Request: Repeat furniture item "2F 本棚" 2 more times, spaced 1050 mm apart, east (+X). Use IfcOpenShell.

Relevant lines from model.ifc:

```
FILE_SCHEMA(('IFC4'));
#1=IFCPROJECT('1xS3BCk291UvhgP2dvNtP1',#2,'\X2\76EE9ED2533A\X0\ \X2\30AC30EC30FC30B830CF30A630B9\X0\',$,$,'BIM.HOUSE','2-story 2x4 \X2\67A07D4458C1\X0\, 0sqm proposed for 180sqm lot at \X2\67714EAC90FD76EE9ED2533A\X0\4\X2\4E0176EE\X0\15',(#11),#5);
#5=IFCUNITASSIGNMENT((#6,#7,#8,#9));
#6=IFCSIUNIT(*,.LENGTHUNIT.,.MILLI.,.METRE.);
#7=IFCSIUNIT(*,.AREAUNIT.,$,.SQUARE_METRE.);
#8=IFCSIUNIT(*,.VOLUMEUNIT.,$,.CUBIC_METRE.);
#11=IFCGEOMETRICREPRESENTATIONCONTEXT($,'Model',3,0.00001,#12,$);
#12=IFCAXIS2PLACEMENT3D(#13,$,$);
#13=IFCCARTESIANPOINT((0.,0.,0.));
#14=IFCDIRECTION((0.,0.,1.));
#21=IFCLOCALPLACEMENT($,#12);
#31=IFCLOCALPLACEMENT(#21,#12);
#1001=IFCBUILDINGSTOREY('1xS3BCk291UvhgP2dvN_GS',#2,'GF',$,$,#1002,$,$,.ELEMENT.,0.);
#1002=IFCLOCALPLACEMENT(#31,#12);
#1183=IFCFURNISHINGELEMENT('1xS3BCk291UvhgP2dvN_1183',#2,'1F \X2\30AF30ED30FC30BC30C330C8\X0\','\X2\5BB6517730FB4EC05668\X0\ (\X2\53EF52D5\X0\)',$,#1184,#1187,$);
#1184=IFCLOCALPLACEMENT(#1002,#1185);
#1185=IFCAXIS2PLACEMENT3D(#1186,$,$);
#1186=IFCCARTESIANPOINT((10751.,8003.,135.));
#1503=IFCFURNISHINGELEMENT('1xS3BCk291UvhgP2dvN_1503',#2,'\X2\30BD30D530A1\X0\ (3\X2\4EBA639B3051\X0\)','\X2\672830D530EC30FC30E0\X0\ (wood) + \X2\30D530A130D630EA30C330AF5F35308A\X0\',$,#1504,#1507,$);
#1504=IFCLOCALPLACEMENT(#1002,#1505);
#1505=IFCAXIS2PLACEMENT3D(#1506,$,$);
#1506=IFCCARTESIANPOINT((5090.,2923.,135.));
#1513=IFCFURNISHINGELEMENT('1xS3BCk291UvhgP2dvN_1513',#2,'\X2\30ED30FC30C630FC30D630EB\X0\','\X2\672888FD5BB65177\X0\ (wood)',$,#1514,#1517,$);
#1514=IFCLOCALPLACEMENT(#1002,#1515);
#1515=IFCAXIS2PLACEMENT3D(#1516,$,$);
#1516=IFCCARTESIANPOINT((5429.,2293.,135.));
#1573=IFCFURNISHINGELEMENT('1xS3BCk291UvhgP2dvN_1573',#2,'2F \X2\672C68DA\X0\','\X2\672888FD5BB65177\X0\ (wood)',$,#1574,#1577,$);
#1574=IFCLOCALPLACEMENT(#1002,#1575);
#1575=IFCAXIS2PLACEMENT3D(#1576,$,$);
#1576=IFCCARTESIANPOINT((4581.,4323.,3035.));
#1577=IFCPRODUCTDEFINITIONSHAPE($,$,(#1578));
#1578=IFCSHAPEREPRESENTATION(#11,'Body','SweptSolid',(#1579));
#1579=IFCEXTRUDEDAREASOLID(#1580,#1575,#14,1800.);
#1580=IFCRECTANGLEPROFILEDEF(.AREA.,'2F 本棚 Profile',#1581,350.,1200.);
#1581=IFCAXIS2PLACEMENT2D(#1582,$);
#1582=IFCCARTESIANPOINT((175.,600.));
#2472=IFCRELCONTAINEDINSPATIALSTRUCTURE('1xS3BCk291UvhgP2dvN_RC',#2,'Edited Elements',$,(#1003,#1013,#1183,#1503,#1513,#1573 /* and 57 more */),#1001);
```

```python
import numpy as np
import ifcopenshell
import ifcopenshell.api.geometry
import ifcopenshell.api.root
import ifcopenshell.util.element
import ifcopenshell.util.placement

model = ifcopenshell.open("model.ifc")


def reuse_history(source, copy):
    """copy_class also copies each property set's owner history, people and application; keep the originals."""
    for rel in copy.IsDefinedBy:
        if rel.is_a("IfcRelDefinesByProperties") and (history := rel.RelatingPropertyDefinition.OwnerHistory):
            rel.RelatingPropertyDefinition.OwnerHistory = source.OwnerHistory
            ifcopenshell.util.element.remove_deep2(model, history)


source = model.by_guid("1xS3BCk291UvhgP2dvN_1573")
base = ifcopenshell.util.placement.get_local_placement(source.ObjectPlacement)
step = np.array([1.0, 0.0, 0.0]) * 1050.0

for i in range(1, 3):
    copy = ifcopenshell.api.root.copy_class(model, product=source)
    copy.Representation = ifcopenshell.util.element.copy_deep(
        model, source.Representation, exclude=["IfcGeometricRepresentationContext", "IfcRepresentationMap"]
    )
    reuse_history(source, copy)
    matrix = base.copy()
    matrix[:3, 3] += i * step
    print("added at", matrix[:3, 3].round(3) + 0.0)
    ifcopenshell.api.geometry.edit_object_placement(model, product=copy, matrix=matrix, is_si=False)

model.write("model_v2.ifc")
```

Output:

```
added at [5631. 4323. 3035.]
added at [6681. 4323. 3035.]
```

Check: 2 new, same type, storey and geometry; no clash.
